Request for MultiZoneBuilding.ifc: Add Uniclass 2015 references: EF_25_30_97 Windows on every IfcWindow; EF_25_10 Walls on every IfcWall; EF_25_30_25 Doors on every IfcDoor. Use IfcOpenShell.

First a look at what the model holds.

```python
import ifcopenshell

model = ifcopenshell.open("MultiZoneBuilding.ifc")
print(model.schema)
print("classifications:", [c.Name for c in model.by_type("IfcClassification")])
for ifc_class in ("IfcDoor", "IfcRoof", "IfcStair", "IfcWall", "IfcWindow"):
    print(ifc_class, len(model.by_type(ifc_class)))
```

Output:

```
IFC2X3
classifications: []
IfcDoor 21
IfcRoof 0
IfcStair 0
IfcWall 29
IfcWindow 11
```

```python
import ifcopenshell
import ifcopenshell.api.classification

model = ifcopenshell.open("MultiZoneBuilding.ifc")

# IFC2X3 requires Source and Edition and has no link from the project to the system.
system = model.create_entity("IfcClassification", Source="NBS", Edition="2015", Name="Uniclass 2015")

codes = {
    "IfcWindow": ("EF_25_30_97", "Windows"),
    "IfcWall": ("EF_25_10", "Walls"),
    "IfcDoor": ("EF_25_30_25", "Doors"),
}
for ifc_class, (code, name) in codes.items():
    products = model.by_type(ifc_class)
    ifcopenshell.api.classification.add_reference(
        model, products=products, classification=system, identification=code, name=name
    )
    print(code, len(products))

model.write("MultiZoneBuilding_updated.ifc")
```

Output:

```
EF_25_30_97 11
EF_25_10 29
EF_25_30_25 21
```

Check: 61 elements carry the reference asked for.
